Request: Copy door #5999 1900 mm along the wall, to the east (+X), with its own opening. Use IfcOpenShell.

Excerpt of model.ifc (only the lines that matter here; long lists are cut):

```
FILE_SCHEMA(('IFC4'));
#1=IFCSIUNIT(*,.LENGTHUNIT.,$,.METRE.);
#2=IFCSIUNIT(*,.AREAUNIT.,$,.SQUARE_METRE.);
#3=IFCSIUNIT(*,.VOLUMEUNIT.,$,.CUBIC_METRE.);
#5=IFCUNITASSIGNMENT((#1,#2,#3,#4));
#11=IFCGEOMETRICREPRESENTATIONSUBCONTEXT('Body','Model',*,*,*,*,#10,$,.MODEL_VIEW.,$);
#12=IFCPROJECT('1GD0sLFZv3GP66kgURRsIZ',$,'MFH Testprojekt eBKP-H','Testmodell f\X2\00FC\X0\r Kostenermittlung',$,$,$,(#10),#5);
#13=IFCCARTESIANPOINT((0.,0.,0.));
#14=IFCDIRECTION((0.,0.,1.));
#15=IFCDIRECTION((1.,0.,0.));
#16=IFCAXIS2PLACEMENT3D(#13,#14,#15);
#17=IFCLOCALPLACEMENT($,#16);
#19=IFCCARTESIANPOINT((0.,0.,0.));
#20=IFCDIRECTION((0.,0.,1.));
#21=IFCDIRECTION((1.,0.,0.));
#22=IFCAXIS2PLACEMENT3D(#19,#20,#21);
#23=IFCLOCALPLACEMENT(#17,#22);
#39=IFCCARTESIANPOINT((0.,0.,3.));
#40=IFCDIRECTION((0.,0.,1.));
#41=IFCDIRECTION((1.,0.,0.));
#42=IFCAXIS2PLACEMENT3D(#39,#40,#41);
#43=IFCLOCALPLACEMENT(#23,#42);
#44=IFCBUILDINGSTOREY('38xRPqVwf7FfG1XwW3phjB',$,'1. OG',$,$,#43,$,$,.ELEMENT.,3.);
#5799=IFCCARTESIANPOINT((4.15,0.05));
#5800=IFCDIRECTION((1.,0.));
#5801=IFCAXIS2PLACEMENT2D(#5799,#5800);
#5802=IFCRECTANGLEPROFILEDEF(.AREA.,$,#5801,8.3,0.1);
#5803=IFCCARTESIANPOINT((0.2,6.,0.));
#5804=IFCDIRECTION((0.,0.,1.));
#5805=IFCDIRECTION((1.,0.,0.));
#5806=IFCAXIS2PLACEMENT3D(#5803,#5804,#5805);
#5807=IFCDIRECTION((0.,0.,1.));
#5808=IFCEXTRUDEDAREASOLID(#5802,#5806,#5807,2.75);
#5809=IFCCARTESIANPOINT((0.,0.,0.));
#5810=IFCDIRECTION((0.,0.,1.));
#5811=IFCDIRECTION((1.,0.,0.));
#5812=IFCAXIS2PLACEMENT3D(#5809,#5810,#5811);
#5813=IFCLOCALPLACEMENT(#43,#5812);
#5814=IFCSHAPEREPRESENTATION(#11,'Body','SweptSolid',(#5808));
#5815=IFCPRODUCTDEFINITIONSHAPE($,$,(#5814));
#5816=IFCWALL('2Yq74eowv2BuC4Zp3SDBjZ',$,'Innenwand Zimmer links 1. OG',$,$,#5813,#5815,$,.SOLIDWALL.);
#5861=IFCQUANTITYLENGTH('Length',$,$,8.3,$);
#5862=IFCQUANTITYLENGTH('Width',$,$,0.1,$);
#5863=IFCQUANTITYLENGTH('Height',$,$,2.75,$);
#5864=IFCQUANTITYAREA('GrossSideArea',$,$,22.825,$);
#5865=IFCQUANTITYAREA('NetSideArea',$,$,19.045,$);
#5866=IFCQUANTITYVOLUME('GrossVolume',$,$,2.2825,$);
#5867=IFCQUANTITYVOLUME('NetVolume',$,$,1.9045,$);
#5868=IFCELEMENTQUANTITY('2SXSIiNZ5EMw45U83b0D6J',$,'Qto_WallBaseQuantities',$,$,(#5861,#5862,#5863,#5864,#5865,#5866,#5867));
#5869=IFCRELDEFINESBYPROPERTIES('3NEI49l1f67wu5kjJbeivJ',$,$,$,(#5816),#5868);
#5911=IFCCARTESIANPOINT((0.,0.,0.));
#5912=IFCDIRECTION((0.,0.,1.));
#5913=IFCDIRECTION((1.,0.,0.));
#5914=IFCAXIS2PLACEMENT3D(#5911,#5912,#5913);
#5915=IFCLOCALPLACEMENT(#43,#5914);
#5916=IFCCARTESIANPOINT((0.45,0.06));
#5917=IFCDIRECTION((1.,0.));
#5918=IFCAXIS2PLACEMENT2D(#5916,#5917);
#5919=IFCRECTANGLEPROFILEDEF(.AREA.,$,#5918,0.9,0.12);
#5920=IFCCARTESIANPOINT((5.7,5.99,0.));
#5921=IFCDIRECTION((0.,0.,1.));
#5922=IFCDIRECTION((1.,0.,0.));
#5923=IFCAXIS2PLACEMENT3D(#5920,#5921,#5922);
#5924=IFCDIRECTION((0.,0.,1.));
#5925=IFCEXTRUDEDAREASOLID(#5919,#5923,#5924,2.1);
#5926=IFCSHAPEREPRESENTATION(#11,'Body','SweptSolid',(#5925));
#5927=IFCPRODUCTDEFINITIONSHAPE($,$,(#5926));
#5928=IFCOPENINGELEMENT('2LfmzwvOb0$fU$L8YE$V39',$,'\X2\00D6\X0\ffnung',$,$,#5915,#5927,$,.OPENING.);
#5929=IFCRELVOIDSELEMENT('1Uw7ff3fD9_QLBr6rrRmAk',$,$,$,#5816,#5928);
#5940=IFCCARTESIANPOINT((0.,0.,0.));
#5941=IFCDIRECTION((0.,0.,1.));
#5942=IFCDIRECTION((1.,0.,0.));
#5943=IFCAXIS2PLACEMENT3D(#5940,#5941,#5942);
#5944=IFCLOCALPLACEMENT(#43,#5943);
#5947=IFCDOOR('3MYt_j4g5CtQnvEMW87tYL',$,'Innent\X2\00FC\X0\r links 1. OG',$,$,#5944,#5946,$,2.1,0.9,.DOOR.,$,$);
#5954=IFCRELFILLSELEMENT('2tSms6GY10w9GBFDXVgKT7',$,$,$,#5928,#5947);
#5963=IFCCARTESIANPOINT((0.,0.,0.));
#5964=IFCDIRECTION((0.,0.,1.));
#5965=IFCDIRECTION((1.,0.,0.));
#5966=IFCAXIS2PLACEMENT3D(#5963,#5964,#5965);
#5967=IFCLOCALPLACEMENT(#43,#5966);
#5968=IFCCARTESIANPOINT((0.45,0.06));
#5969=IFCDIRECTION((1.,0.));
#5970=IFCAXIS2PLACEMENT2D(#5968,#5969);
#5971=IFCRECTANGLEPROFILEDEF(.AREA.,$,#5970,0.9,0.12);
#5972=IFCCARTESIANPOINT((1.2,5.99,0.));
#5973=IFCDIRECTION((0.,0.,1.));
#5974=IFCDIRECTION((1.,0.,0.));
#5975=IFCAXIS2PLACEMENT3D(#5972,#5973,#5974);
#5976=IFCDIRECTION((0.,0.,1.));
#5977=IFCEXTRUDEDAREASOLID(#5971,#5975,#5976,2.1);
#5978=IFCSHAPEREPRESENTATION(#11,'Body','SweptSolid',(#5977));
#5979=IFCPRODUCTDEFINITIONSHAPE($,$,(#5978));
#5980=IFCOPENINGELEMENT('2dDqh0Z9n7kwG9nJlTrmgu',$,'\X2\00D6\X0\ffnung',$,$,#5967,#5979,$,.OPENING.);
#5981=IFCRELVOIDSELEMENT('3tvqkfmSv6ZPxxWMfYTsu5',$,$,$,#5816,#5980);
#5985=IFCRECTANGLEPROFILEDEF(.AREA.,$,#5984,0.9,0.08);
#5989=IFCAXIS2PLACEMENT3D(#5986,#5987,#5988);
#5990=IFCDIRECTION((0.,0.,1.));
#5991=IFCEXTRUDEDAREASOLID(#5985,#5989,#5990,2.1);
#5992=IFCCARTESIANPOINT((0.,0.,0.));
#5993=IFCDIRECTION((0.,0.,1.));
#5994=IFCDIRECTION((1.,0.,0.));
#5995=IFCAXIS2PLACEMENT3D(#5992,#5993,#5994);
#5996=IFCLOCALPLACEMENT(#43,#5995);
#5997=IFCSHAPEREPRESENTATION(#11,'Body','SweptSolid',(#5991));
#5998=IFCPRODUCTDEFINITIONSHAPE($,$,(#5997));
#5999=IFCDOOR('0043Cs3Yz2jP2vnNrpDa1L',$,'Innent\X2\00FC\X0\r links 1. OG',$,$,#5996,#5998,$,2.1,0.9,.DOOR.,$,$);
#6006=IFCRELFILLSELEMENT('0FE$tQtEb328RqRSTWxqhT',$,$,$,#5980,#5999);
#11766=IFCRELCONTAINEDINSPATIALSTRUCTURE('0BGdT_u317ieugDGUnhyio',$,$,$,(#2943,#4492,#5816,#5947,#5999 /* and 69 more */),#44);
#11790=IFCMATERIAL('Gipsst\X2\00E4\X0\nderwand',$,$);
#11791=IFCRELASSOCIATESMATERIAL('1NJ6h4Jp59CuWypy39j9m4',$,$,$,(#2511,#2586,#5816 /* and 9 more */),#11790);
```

```python
import ifcopenshell
import ifcopenshell.api.feature
import ifcopenshell.api.geometry
import ifcopenshell.api.pset
import ifcopenshell.api.root
import ifcopenshell.geom
import ifcopenshell.util.element
import ifcopenshell.util.placement
import ifcopenshell.util.shape
import ifcopenshell.util.unit

model = ifcopenshell.open("model.ifc")
area_scale = ifcopenshell.util.unit.calculate_unit_scale(model, "AREAUNIT")
volume_scale = ifcopenshell.util.unit.calculate_unit_scale(model, "VOLUMEUNIT")
settings = ifcopenshell.geom.settings()


def volume(element):
    """Net volume in cubic metres, openings subtracted."""
    shape = ifcopenshell.geom.create_shape(settings, element)
    return ifcopenshell.util.shape.get_volume(shape.geometry)


door = model.by_guid("0043Cs3Yz2jP2vnNrpDa1L")
opening = door.FillsVoids[0].RelatingOpeningElement
wall = opening.VoidsElements[0].RelatingBuildingElement
before = volume(wall)
shift = ifcopenshell.util.placement.get_local_placement(wall.ObjectPlacement)[:3, 0] * 1.9

# copy_class copies the void relationship, type, container and properties, but no geometry.
new_opening = ifcopenshell.api.root.copy_class(model, product=opening)
new_opening.Representation = ifcopenshell.util.element.copy_deep(
    model, opening.Representation, exclude=["IfcGeometricRepresentationContext", "IfcRepresentationMap"]
)
new_door = ifcopenshell.api.root.copy_class(model, product=door)
new_door.Representation = ifcopenshell.util.element.copy_deep(
    model, door.Representation, exclude=["IfcGeometricRepresentationContext", "IfcRepresentationMap"]
)
ifcopenshell.api.feature.add_filling(model, opening=new_opening, element=new_door)

for old, new in ((opening, new_opening), (door, new_door)):
    matrix = ifcopenshell.util.placement.get_local_placement(old.ObjectPlacement)
    matrix[:3, 3] += shift
    ifcopenshell.api.geometry.edit_object_placement(model, product=new, matrix=matrix, is_si=False)

after = volume(wall)
thickness = 0.1  # wall thickness in metres

# Update the wall's stored quantities.
qto = model.by_id(ifcopenshell.util.element.get_pset(wall, "Qto_WallBaseQuantities", should_inherit=False)["id"])
ifcopenshell.api.pset.edit_qto(model, qto=qto, properties={
    "NetSideArea": after / thickness / area_scale,
    "NetVolume": after / volume_scale,
})

print(f"wall volume {before:.3f} -> {after:.3f} m3")

model.write("model_edited.ifc")
```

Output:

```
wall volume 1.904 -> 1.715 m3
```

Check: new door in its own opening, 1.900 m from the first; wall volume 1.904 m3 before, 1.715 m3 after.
